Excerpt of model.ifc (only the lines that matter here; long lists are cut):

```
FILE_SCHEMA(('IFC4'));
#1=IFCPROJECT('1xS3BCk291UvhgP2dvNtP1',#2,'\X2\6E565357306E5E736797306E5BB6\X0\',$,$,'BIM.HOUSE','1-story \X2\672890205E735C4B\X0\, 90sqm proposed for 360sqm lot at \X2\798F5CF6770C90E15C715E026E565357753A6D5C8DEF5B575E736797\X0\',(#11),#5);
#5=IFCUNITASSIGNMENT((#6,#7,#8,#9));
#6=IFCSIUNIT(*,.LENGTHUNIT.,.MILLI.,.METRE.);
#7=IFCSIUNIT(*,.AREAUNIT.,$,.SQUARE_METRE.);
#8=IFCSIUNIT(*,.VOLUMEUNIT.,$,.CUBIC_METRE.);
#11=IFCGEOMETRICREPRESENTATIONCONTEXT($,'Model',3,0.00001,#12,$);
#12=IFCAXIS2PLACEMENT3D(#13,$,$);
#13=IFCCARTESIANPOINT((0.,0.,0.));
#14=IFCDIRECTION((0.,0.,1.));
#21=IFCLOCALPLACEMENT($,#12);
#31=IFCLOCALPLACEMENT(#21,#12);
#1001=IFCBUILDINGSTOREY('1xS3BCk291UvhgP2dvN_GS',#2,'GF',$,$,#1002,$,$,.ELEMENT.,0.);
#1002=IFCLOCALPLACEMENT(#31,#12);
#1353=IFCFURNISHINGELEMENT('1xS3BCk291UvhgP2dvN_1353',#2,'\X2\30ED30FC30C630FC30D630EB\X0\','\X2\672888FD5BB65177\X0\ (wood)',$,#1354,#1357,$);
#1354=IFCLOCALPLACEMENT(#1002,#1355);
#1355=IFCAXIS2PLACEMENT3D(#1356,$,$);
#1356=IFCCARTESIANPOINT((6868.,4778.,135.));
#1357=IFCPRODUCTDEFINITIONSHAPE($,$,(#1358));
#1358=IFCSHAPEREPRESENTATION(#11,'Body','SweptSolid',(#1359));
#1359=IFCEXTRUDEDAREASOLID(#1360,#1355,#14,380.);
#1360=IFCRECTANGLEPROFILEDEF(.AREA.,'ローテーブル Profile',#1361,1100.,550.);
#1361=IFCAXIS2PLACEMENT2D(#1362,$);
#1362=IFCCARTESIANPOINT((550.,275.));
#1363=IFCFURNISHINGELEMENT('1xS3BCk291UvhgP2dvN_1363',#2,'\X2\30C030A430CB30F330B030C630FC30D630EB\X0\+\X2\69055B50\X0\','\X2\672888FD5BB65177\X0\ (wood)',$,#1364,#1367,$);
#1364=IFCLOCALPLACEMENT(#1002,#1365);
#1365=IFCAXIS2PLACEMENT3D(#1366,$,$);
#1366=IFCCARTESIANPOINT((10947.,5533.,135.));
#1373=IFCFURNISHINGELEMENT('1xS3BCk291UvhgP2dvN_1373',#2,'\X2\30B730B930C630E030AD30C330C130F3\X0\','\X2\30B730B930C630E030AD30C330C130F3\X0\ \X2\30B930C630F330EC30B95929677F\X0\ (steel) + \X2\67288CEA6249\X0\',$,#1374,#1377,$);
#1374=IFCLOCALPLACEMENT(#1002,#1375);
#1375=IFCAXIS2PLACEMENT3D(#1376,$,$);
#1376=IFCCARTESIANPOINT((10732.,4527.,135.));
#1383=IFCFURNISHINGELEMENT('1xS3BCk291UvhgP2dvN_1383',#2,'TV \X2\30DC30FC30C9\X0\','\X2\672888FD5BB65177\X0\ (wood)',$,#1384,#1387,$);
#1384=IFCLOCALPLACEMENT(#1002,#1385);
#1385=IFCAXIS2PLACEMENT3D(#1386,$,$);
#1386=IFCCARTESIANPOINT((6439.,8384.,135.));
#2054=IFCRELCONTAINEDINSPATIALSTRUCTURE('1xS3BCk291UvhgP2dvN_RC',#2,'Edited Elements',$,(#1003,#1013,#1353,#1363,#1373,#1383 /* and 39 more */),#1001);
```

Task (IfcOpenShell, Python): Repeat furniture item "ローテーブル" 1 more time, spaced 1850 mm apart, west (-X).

```python
import numpy as np
import ifcopenshell
import ifcopenshell.api.geometry
import ifcopenshell.api.root
import ifcopenshell.util.element
import ifcopenshell.util.placement

model = ifcopenshell.open("model.ifc")


def reuse_history(source, copy):
    """copy_class also copies each property set's owner history, people and application; keep the originals."""
    for rel in copy.IsDefinedBy:
        if rel.is_a("IfcRelDefinesByProperties") and (history := rel.RelatingPropertyDefinition.OwnerHistory):
            rel.RelatingPropertyDefinition.OwnerHistory = source.OwnerHistory
            ifcopenshell.util.element.remove_deep2(model, history)


source = model.by_guid("1xS3BCk291UvhgP2dvN_1353")
base = ifcopenshell.util.placement.get_local_placement(source.ObjectPlacement)
step = np.array([-1.0, 0.0, 0.0]) * 1850.0

for i in range(1, 2):
    copy = ifcopenshell.api.root.copy_class(model, product=source)
    copy.Representation = ifcopenshell.util.element.copy_deep(
        model, source.Representation, exclude=["IfcGeometricRepresentationContext", "IfcRepresentationMap"]
    )
    reuse_history(source, copy)
    matrix = base.copy()
    matrix[:3, 3] += i * step
    print("added at", matrix[:3, 3].round(3) + 0.0)
    ifcopenshell.api.geometry.edit_object_placement(model, product=copy, matrix=matrix, is_si=False)

model.write("model-out.ifc")
```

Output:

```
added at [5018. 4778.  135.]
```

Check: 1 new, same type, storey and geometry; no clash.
